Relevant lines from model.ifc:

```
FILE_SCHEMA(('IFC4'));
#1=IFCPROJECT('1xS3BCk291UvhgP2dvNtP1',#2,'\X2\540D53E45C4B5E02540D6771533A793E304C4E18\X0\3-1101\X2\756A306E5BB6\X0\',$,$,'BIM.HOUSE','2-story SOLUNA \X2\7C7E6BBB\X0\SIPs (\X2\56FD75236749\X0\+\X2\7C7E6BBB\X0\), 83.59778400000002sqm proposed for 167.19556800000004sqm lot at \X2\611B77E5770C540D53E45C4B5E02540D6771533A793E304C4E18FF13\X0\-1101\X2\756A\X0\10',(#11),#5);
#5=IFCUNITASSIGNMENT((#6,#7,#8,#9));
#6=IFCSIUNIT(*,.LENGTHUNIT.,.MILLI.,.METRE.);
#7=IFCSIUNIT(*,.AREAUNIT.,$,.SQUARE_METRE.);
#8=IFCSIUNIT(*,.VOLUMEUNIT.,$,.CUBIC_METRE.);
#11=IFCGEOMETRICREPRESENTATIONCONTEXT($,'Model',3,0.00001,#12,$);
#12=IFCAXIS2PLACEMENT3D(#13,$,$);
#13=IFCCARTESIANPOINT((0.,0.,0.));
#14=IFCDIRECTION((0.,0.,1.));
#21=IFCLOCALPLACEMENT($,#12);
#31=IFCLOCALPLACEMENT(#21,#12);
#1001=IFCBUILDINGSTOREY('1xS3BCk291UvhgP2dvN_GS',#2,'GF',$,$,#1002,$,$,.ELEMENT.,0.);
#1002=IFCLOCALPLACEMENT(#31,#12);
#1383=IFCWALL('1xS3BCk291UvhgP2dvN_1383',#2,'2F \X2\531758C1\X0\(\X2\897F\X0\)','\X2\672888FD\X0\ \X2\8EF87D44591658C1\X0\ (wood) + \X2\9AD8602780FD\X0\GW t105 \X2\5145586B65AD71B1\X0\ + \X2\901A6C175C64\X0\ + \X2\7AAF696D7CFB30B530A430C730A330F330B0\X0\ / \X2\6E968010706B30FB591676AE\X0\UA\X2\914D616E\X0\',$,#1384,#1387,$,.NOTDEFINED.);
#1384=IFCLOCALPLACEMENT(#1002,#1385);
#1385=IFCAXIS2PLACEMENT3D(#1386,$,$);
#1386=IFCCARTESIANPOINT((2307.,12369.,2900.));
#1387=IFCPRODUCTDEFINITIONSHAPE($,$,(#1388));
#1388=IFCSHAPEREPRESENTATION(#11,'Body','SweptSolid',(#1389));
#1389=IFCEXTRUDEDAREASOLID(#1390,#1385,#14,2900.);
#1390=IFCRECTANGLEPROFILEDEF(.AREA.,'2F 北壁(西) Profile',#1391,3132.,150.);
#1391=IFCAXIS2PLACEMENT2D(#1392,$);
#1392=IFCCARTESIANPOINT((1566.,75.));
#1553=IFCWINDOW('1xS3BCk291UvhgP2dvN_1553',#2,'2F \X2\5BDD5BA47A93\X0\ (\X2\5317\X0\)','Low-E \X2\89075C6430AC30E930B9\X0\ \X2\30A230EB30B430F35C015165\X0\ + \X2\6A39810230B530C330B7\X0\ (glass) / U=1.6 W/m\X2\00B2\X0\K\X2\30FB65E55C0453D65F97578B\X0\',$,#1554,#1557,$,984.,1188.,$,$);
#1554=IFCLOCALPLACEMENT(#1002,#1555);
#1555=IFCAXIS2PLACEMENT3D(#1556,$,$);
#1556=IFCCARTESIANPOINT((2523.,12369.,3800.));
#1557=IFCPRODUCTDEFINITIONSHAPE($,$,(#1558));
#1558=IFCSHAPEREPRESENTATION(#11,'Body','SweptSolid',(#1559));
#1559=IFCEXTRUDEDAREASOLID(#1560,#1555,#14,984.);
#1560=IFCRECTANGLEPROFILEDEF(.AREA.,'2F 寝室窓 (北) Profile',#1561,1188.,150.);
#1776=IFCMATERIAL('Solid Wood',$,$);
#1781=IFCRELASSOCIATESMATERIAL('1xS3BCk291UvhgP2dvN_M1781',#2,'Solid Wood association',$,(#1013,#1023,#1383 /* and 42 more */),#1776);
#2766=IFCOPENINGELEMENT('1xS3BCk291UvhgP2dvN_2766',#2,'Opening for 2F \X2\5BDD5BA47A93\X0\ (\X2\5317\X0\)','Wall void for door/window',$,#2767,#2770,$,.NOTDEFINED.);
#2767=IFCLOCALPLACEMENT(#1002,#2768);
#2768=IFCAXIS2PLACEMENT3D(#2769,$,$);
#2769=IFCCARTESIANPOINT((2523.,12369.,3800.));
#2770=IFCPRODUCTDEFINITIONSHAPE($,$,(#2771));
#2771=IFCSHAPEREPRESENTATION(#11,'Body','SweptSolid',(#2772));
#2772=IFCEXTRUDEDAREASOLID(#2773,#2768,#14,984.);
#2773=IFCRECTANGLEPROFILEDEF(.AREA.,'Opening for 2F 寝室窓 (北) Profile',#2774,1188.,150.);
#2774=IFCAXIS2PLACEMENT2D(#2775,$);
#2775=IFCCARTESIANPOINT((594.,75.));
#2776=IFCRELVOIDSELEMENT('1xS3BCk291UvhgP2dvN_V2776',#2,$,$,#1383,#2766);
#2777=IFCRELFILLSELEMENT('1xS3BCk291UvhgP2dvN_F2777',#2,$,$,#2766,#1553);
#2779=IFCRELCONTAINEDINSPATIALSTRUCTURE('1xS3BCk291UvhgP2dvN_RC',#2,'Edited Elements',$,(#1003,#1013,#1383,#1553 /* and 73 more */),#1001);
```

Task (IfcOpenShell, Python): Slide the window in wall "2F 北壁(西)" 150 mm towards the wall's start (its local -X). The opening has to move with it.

```python
import ifcopenshell
import ifcopenshell.api.geometry
import ifcopenshell.util.placement
import ifcopenshell.util.unit

model = ifcopenshell.open("model.ifc")
unit_scale = ifcopenshell.util.unit.calculate_unit_scale(model)

window = model.by_guid("1xS3BCk291UvhgP2dvN_1553")
opening = window.FillsVoids[0].RelatingOpeningElement
wall = opening.VoidsElements[0].RelatingBuildingElement

wall_matrix = ifcopenshell.util.placement.get_local_placement(wall.ObjectPlacement)
shift = wall_matrix[:3, 0] * -0.15 / unit_scale
before = ifcopenshell.util.placement.get_local_placement(window.ObjectPlacement)[:3, 3].copy()

# The window is not placed relative to its opening, so move both.
for product in (opening, window):
    matrix = ifcopenshell.util.placement.get_local_placement(product.ObjectPlacement)
    matrix[:3, 3] += shift
    ifcopenshell.api.geometry.edit_object_placement(model, product=product, matrix=matrix, is_si=False)

after = ifcopenshell.util.placement.get_local_placement(window.ObjectPlacement)[:3, 3]
print("window moved by", (after - before).round(3) + 0.0)

model.write("model-out.ifc")
```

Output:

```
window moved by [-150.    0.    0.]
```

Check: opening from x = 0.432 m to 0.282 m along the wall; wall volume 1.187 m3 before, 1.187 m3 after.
